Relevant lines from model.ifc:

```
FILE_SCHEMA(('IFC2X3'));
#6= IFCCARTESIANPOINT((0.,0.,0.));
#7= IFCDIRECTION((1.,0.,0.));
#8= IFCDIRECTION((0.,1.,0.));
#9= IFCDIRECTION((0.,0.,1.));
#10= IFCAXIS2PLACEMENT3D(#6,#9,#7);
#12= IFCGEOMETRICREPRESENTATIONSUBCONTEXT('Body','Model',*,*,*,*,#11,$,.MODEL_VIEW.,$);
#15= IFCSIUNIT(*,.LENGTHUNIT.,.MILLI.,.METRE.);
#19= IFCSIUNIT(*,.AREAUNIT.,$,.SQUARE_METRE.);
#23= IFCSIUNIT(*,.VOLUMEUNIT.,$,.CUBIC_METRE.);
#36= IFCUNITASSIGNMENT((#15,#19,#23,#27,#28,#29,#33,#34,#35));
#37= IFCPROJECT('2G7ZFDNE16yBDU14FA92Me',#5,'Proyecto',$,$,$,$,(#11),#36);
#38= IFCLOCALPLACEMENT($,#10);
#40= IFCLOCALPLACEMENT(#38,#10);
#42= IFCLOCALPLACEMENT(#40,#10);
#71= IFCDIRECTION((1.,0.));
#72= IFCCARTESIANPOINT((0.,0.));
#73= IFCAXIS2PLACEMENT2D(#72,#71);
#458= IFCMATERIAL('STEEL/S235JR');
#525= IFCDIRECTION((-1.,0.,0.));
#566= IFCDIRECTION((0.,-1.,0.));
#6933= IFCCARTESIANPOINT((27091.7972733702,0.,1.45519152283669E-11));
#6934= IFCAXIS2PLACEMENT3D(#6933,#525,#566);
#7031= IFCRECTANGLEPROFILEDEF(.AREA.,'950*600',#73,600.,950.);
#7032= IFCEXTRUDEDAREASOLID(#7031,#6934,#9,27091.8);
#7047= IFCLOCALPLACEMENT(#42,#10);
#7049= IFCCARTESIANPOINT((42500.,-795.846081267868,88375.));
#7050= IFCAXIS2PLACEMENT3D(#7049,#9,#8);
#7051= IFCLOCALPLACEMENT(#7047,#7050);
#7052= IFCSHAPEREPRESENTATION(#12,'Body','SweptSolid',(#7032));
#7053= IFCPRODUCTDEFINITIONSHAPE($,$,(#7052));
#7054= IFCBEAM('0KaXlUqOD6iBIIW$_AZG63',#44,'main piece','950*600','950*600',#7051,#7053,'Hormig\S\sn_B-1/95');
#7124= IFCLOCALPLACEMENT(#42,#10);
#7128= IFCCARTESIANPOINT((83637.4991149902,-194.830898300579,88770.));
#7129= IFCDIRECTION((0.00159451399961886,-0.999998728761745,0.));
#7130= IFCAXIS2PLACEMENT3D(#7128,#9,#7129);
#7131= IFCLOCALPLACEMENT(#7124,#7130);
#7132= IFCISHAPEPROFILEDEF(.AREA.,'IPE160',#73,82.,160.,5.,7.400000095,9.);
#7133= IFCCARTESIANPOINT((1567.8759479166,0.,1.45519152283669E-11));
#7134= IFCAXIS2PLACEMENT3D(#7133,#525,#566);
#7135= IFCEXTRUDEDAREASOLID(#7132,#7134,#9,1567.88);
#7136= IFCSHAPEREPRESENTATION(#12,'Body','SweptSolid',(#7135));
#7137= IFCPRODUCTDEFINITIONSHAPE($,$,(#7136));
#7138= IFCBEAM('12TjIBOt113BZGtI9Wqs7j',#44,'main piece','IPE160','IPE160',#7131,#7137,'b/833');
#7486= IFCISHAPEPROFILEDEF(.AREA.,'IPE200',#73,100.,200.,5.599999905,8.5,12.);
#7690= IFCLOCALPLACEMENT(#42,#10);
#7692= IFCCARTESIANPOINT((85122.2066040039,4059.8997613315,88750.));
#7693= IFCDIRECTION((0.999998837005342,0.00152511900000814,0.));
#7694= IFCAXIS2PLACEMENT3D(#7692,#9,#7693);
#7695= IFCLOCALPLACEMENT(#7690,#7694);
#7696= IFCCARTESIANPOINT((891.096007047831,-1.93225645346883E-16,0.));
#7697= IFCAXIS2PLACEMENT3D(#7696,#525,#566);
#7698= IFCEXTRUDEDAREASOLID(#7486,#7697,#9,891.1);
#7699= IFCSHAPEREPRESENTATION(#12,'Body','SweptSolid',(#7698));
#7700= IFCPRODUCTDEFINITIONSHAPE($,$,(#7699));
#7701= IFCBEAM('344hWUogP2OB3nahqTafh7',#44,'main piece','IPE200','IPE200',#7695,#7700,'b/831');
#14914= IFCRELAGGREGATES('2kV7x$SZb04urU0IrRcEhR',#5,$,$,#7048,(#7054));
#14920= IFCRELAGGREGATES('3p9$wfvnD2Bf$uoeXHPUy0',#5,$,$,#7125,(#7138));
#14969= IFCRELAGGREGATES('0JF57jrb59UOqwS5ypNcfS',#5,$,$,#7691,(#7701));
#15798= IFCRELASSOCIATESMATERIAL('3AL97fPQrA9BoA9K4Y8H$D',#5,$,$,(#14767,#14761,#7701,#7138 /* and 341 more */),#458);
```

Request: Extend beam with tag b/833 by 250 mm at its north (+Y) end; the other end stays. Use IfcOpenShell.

```python
import ifcopenshell
import ifcopenshell.util.representation
import ifcopenshell.util.unit

model = ifcopenshell.open("model.ifc")
unit_scale = ifcopenshell.util.unit.calculate_unit_scale(model)

member = model.by_guid("12TjIBOt113BZGtI9Wqs7j")
change = 0.25 / unit_scale

# The extrusion runs towards the end named, so only its depth changes.
body = ifcopenshell.util.representation.get_representation(member, "Model", "Body")
solid = body.Items[0]
old_length = solid.Depth
solid.Depth += change

print(f"length {old_length:g} -> {solid.Depth:g}")

model.write("model-out.ifc")
```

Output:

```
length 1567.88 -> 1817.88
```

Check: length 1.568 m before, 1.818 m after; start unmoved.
